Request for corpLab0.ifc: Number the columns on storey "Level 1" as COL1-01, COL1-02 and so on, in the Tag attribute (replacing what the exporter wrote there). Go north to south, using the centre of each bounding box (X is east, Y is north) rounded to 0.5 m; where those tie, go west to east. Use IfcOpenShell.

First a look at what the model holds.

```python
import ifcopenshell
import ifcopenshell.util.element
import ifcopenshell.util.placement

model = ifcopenshell.open("corpLab0.ifc")
print(model.schema)
storey = next(s for s in model.by_type("IfcBuildingStorey") if s.Name == "Level 1")
columns = [e for e in ifcopenshell.util.element.get_decomposition(storey) if e.is_a("IfcColumn")]
for e in sorted(columns, key=lambda e: e.id()):
    origin = ifcopenshell.util.placement.get_local_placement(e.ObjectPlacement)[:3, 3]
    print(e.id(), e.Tag, e.Name, origin.round(2) + 0.0, sep=" | ")
```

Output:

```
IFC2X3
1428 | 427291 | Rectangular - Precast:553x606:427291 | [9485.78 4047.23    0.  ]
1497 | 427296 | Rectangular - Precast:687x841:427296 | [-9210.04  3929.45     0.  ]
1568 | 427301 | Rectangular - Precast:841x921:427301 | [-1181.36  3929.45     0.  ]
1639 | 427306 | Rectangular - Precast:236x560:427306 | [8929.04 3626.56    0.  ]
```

```python
import ifcopenshell
import ifcopenshell.geom
import ifcopenshell.util.element
import ifcopenshell.util.shape

model = ifcopenshell.open("corpLab0.ifc")
settings = ifcopenshell.geom.settings()
settings.set("use-world-coords", True)


def centre(element):
    shape = ifcopenshell.geom.create_shape(settings, element)
    return ifcopenshell.util.shape.get_bbox_centroid(shape.geometry)


storey = next(s for s in model.by_type("IfcBuildingStorey") if s.Name == "Level 1")
columns = [e for e in ifcopenshell.util.element.get_decomposition(storey) if e.is_a("IfcColumn")]

# Insertion points can sit at a corner or the storey origin, so sort by the geometry (in metres).
centres = {e: centre(e) for e in columns}
columns.sort(key=lambda e: (-round(centres[e][1] / 0.5), centres[e][0]))

for i, e in enumerate(columns, start=1):
    number = f"COL1-{i:02d}"
    e.Tag = number
    print(e.id(), number)

model.write("corpLab0_rev.ifc")
```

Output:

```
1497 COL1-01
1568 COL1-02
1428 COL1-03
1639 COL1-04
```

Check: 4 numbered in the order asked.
